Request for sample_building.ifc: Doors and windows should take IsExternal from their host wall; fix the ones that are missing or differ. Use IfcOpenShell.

First a look at what the model holds.

```python
import ifcopenshell
import ifcopenshell.util.element

model = ifcopenshell.open("sample_building.ifc")
print(model.schema)
seen = {}
for e in model.by_type("IfcDoor") + model.by_type("IfcWindow"):
    if not e.FillsVoids:
        continue
    host = e.FillsVoids[0].RelatingOpeningElement.VoidsElements[0].RelatingBuildingElement
    own = ifcopenshell.util.element.get_pset(e, f"Pset_{e.is_a()[3:].removesuffix('StandardCase')}Common", "IsExternal")
    wall = ifcopenshell.util.element.get_pset(host, "Pset_WallCommon", "IsExternal")
    seen[e.is_a(), own, wall] = seen.get((e.is_a(), own, wall), 0) + 1
for (cls, own, wall), count in sorted(seen.items(), key=str):
    print(count, cls, "IsExternal:", own, "| host wall:", wall)
```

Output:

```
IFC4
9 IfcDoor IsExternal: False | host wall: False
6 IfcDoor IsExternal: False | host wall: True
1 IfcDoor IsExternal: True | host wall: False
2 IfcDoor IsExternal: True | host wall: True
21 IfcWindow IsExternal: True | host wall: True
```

```python
import ifcopenshell
import ifcopenshell.api.pset
import ifcopenshell.util.element

model = ifcopenshell.open("sample_building.ifc")

count = 0
for ifc_class, pset_name in (("IfcDoor", "Pset_DoorCommon"), ("IfcWindow", "Pset_WindowCommon")):
    for e in model.by_type(ifc_class):
        if not e.FillsVoids:
            continue
        host = e.FillsVoids[0].RelatingOpeningElement.VoidsElements[0].RelatingBuildingElement
        external = ifcopenshell.util.element.get_pset(host, "Pset_WallCommon", "IsExternal")
        if external is None or ifcopenshell.util.element.get_pset(e, pset_name, "IsExternal") == external:
            continue
        pset = ifcopenshell.api.pset.add_pset(model, product=e, name=pset_name)
        ifcopenshell.api.pset.edit_pset(model, pset=pset, properties={"IsExternal": external})
        count += 1

print(count, "updated")

model.write("sample_building-out.ifc")
```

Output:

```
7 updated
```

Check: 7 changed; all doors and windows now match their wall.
